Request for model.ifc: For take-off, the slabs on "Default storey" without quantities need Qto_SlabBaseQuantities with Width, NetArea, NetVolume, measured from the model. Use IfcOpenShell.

First a look at what the model holds.

```python
import ifcopenshell
import ifcopenshell.util.element
import ifcopenshell.util.unit

model = ifcopenshell.open("model.ifc")
print(model.schema)
for unit_type in ("LENGTHUNIT", "AREAUNIT", "VOLUMEUNIT"):
    print(unit_type, ifcopenshell.util.unit.calculate_unit_scale(model, unit_type))
storey = next(s for s in model.by_type("IfcBuildingStorey") if s.Name == "Default storey")
slabs = [e for e in ifcopenshell.util.element.get_decomposition(storey) if e.is_a("IfcSlab")]
for e in sorted(slabs, key=lambda e: e.id()):
    print(e.id(), e.is_a(), e.Name, list(ifcopenshell.util.element.get_psets(e, qtos_only=True)), sep=" | ")
```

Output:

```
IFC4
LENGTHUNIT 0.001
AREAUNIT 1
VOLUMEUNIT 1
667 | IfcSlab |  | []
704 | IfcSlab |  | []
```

```python
import ifcopenshell
import ifcopenshell.api.pset
import ifcopenshell.geom
import ifcopenshell.util.element
import ifcopenshell.util.shape
import ifcopenshell.util.unit

model = ifcopenshell.open("model.ifc")
unit_scale = ifcopenshell.util.unit.calculate_unit_scale(model)
area_scale = ifcopenshell.util.unit.calculate_unit_scale(model, "AREAUNIT")
volume_scale = ifcopenshell.util.unit.calculate_unit_scale(model, "VOLUMEUNIT")
settings = ifcopenshell.geom.settings()

storey = next(s for s in model.by_type("IfcBuildingStorey") if s.Name == "Default storey")
slabs = [e for e in ifcopenshell.util.element.get_decomposition(storey) if e.is_a("IfcSlab")]

for e in sorted(slabs, key=lambda e: e.id()):
    if ifcopenshell.util.element.get_psets(e, qtos_only=True, should_inherit=False):
        continue
    # Geometry comes back in metres, in the element's own axes.
    shape = ifcopenshell.geom.create_shape(settings, e)
    values = {
        "Width": ifcopenshell.util.shape.get_z(shape.geometry) / unit_scale,
        "NetArea": ifcopenshell.util.shape.get_footprint_area(shape.geometry) / area_scale,
        "NetVolume": ifcopenshell.util.shape.get_volume(shape.geometry) / volume_scale,
    }
    qto = ifcopenshell.api.pset.add_qto(model, product=e, name="Qto_SlabBaseQuantities")
    ifcopenshell.api.pset.edit_qto(model, qto=qto, properties=values)
    print(e.id(), {k: round(v, 3) for k, v in values.items()})

model.write("model_edited.ifc")
```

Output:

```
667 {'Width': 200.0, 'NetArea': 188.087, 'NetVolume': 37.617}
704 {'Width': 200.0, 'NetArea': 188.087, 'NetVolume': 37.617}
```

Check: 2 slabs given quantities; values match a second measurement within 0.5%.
